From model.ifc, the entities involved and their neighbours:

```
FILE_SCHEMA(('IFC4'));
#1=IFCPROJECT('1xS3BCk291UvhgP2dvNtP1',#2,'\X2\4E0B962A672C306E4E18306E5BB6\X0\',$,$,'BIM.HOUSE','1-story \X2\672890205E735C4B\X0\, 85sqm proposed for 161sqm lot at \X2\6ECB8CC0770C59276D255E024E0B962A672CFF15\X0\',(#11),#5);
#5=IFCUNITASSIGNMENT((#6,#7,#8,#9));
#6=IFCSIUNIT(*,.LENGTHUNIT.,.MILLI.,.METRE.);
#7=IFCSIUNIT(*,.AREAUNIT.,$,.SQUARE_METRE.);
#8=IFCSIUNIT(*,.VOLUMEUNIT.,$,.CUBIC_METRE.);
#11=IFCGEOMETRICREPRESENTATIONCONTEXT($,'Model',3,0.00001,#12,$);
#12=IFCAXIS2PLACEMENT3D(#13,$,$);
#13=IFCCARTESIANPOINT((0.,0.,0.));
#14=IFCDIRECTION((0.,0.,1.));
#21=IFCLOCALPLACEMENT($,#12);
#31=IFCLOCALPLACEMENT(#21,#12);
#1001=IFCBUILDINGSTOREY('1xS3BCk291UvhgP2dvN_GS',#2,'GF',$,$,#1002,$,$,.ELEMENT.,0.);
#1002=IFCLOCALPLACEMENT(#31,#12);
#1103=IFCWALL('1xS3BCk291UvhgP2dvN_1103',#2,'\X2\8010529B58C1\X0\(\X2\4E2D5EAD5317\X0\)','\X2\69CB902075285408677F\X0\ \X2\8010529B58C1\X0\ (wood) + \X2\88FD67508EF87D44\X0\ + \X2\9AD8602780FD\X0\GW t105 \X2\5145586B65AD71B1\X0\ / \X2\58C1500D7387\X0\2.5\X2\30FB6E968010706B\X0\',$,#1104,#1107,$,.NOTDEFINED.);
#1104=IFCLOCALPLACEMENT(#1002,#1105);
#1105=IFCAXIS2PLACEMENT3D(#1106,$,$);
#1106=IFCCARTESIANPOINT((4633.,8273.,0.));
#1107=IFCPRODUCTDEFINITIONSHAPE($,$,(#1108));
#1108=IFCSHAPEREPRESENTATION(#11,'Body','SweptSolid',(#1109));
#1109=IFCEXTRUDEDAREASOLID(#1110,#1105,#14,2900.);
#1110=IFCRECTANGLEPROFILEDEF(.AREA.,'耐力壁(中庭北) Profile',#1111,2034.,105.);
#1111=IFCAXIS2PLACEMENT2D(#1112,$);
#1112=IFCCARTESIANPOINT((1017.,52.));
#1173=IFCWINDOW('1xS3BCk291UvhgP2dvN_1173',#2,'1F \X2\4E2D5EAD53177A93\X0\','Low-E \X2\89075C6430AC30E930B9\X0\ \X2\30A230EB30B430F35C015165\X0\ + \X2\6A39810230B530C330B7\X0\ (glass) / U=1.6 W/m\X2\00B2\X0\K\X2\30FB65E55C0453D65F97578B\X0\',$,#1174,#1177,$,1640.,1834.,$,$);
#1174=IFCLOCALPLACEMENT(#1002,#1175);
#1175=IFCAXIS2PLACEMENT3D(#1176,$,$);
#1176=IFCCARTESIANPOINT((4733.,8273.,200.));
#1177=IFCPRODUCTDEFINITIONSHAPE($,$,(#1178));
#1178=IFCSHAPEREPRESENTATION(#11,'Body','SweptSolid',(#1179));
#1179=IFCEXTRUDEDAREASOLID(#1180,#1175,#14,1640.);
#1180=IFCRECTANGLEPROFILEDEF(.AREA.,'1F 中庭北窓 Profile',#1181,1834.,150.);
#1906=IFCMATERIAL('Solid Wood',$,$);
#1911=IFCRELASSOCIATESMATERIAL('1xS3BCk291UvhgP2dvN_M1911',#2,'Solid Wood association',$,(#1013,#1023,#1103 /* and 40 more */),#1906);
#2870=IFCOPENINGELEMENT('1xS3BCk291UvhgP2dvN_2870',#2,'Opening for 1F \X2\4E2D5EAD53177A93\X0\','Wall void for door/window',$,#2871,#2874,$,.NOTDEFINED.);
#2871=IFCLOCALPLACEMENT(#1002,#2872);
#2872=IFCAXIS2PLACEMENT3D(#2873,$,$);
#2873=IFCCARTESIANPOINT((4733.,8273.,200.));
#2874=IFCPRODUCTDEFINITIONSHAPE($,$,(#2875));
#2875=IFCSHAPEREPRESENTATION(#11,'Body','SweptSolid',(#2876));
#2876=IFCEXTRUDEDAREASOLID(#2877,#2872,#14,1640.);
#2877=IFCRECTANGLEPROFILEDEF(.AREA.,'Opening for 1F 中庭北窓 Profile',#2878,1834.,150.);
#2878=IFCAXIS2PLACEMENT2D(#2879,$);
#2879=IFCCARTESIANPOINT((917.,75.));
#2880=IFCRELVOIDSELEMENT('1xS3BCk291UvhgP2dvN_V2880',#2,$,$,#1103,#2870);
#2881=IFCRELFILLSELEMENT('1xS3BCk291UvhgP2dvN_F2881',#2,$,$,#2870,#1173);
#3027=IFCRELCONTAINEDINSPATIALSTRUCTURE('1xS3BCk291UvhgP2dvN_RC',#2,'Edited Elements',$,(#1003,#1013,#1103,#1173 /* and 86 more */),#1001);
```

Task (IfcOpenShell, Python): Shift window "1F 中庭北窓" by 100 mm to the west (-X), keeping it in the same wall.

```python
import ifcopenshell
import ifcopenshell.api.geometry
import ifcopenshell.util.placement
import ifcopenshell.util.unit

model = ifcopenshell.open("model.ifc")
unit_scale = ifcopenshell.util.unit.calculate_unit_scale(model)

window = model.by_guid("1xS3BCk291UvhgP2dvN_1173")
opening = window.FillsVoids[0].RelatingOpeningElement
wall = opening.VoidsElements[0].RelatingBuildingElement

wall_matrix = ifcopenshell.util.placement.get_local_placement(wall.ObjectPlacement)
shift = wall_matrix[:3, 0] * -0.1 / unit_scale
before = ifcopenshell.util.placement.get_local_placement(window.ObjectPlacement)[:3, 3].copy()

# The window is not placed relative to its opening, so move both.
for product in (opening, window):
    matrix = ifcopenshell.util.placement.get_local_placement(product.ObjectPlacement)
    matrix[:3, 3] += shift
    ifcopenshell.api.geometry.edit_object_placement(model, product=product, matrix=matrix, is_si=False)

after = ifcopenshell.util.placement.get_local_placement(window.ObjectPlacement)[:3, 3]
print("window moved by", (after - before).round(3) + 0.0)

model.write("model_v2.ifc")
```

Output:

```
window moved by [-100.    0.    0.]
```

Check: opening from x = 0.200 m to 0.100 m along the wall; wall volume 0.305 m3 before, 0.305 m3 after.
